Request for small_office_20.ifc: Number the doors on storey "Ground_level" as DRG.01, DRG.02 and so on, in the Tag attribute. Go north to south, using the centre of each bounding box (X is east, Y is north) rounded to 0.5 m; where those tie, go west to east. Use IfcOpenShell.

First a look at what the model holds.

```python
import ifcopenshell
import ifcopenshell.util.element
import ifcopenshell.util.placement

model = ifcopenshell.open("small_office_20.ifc")
print(model.schema)
storey = next(s for s in model.by_type("IfcBuildingStorey") if s.Name == "Ground_level")
doors = [e for e in ifcopenshell.util.element.get_decomposition(storey) if e.is_a("IfcDoor")]
for e in sorted(doors, key=lambda e: e.id()):
    origin = ifcopenshell.util.placement.get_local_placement(e.ObjectPlacement)[:3, 3]
    print(e.id(), e.Tag, e.Name, origin.round(2) + 0.0, sep=" | ")
```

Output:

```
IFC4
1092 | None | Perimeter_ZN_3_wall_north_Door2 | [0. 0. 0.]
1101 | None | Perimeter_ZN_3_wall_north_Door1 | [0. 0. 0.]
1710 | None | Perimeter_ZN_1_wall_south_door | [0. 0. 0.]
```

```python
import ifcopenshell
import ifcopenshell.geom
import ifcopenshell.util.element
import ifcopenshell.util.shape

model = ifcopenshell.open("small_office_20.ifc")
settings = ifcopenshell.geom.settings()
settings.set("use-world-coords", True)


def centre(element):
    shape = ifcopenshell.geom.create_shape(settings, element)
    return ifcopenshell.util.shape.get_bbox_centroid(shape.geometry)


storey = next(s for s in model.by_type("IfcBuildingStorey") if s.Name == "Ground_level")
doors = [e for e in ifcopenshell.util.element.get_decomposition(storey) if e.is_a("IfcDoor")]

# Insertion points can sit at a corner or the storey origin, so sort by the geometry (in metres).
centres = {e: centre(e) for e in doors}
doors.sort(key=lambda e: (-round(centres[e][1] / 0.5), centres[e][0]))

for i, e in enumerate(doors, start=1):
    number = f"DRG.{i:02d}"
    e.Tag = number
    print(e.id(), number)

model.write("small_office_20_rev.ifc")
```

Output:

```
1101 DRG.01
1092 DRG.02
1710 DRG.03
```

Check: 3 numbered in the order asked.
